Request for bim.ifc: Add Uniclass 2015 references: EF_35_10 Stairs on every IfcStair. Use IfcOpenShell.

First a look at what the model holds.

```python
import ifcopenshell

model = ifcopenshell.open("bim.ifc")
print(model.schema)
print("classifications:", [c.Name for c in model.by_type("IfcClassification")])
for ifc_class in ("IfcDoor", "IfcRoof", "IfcStair", "IfcWall", "IfcWindow"):
    print(ifc_class, len(model.by_type(ifc_class)))
```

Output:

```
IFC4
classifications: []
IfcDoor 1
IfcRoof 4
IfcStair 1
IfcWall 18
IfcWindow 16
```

```python
import ifcopenshell
import ifcopenshell.api.classification

model = ifcopenshell.open("bim.ifc")

system = ifcopenshell.api.classification.add_classification(model, classification="Uniclass 2015")

codes = {
    "IfcStair": ("EF_35_10", "Stairs"),
}
for ifc_class, (code, name) in codes.items():
    products = model.by_type(ifc_class)
    ifcopenshell.api.classification.add_reference(
        model, products=products, classification=system, identification=code, name=name
    )
    print(code, len(products))

model.write("bim-out.ifc")
```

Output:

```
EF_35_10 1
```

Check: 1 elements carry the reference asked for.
